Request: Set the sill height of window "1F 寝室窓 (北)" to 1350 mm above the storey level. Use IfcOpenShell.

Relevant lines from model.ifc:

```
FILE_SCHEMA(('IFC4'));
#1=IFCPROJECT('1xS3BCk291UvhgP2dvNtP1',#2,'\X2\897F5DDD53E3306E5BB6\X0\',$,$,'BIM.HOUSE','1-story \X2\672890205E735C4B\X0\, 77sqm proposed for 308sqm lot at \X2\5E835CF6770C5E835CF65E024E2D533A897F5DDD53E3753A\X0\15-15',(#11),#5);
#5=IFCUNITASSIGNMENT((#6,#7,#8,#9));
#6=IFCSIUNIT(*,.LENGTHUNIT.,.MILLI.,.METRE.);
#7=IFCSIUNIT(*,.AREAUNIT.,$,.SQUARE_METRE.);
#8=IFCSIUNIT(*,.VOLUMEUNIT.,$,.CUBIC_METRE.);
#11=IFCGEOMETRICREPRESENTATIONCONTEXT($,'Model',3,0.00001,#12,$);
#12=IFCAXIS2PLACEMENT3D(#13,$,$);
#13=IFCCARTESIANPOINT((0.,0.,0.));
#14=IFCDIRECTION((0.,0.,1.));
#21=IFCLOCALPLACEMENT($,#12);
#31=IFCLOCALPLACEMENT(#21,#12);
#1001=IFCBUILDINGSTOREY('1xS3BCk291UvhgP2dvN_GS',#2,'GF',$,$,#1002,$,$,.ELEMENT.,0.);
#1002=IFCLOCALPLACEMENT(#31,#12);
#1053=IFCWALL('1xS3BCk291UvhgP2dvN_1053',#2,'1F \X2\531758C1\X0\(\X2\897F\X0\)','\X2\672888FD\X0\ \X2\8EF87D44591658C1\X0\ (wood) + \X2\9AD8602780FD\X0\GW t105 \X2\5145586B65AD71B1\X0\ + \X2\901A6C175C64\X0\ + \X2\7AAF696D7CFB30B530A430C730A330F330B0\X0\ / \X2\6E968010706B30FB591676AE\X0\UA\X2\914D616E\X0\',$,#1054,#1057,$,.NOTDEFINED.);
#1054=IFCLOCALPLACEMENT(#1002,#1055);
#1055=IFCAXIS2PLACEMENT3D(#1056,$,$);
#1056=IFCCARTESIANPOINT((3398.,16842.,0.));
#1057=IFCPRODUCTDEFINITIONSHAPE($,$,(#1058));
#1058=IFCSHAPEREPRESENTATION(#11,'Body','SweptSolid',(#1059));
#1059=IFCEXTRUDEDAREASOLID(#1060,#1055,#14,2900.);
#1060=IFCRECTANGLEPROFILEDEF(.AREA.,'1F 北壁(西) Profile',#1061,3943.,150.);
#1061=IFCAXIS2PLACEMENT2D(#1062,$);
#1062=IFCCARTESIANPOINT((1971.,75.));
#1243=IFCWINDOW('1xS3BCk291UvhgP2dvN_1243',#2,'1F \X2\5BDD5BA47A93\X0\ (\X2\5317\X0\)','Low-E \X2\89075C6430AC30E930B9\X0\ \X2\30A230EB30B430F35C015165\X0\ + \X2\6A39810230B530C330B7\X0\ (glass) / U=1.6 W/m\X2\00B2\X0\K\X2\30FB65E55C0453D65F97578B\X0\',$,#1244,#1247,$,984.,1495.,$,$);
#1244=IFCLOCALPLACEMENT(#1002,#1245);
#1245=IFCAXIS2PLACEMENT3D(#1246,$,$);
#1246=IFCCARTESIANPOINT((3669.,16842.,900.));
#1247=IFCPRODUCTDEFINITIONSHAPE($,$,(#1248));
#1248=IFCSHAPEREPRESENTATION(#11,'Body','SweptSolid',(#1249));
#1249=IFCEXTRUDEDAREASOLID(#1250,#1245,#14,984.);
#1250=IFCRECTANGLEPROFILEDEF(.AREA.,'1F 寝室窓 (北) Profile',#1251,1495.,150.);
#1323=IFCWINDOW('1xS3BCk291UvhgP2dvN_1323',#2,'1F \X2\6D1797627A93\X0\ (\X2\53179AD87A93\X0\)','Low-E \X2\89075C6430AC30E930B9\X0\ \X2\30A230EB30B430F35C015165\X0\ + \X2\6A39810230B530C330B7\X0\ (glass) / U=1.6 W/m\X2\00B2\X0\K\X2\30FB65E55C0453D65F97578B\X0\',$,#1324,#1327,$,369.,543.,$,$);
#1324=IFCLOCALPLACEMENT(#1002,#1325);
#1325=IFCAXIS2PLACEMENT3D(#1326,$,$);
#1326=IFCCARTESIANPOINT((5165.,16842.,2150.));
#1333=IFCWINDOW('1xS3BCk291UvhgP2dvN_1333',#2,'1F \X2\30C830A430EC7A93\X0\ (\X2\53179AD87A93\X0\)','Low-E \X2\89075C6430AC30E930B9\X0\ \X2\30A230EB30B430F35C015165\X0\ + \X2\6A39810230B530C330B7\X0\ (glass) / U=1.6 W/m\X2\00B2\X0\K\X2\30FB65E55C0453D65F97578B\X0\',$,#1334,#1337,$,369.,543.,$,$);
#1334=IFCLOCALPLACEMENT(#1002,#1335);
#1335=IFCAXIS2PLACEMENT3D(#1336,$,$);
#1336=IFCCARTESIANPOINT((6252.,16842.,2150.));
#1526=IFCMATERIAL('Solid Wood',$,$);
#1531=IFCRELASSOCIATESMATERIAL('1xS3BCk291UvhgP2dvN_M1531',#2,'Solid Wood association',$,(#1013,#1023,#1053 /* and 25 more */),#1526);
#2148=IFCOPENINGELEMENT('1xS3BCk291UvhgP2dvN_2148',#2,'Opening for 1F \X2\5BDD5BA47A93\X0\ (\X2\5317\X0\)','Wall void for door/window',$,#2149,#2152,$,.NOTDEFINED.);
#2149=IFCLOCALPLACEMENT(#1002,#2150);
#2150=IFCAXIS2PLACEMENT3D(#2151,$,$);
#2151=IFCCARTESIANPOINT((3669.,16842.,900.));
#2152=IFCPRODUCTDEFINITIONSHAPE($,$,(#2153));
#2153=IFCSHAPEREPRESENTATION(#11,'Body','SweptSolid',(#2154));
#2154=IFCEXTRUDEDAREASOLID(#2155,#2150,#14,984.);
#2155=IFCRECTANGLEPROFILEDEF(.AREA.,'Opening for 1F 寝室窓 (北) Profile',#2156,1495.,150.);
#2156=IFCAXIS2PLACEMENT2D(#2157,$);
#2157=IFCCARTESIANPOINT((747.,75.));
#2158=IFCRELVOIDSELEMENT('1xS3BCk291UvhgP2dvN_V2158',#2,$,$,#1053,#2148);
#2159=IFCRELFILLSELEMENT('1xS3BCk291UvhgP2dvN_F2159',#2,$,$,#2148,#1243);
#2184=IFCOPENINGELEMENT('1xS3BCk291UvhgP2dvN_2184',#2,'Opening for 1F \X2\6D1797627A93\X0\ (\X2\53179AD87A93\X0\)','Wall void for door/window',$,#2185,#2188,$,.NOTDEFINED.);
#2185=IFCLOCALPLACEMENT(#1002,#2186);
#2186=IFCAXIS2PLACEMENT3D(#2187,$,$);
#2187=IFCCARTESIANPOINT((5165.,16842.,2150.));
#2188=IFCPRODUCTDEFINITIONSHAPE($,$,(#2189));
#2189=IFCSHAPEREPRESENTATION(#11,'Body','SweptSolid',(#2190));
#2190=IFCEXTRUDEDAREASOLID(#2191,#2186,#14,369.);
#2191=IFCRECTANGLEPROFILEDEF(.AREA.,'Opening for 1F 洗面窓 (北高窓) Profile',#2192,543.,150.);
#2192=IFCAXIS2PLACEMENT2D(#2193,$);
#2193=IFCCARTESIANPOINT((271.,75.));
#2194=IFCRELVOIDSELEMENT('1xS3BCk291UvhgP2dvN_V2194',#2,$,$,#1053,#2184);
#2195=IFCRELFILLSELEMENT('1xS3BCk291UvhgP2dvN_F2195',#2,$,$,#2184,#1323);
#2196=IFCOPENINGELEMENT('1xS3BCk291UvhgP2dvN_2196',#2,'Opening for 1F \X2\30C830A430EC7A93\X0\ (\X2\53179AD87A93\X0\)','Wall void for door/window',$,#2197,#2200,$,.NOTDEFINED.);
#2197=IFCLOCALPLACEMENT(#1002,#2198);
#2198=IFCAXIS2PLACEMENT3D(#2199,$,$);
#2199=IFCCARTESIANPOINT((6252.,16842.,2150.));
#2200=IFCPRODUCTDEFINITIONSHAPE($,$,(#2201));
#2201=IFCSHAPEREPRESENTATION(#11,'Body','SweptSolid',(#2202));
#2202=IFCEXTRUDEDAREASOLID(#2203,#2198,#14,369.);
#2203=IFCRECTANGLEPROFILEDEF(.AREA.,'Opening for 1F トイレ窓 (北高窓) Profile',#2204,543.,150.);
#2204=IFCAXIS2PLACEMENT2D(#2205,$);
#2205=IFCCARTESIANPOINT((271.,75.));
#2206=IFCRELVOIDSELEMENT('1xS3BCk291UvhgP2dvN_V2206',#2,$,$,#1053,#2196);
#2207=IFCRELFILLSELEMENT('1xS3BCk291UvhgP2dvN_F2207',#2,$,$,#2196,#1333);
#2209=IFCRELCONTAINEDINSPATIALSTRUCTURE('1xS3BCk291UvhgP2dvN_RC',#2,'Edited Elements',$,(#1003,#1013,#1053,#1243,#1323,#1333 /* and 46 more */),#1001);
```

```python
import numpy as np
import ifcopenshell
import ifcopenshell.api.geometry
import ifcopenshell.geom
import ifcopenshell.util.element
import ifcopenshell.util.placement
import ifcopenshell.util.shape
import ifcopenshell.util.unit

model = ifcopenshell.open("model.ifc")
unit_scale = ifcopenshell.util.unit.calculate_unit_scale(model)

window = model.by_id(1243)
opening = window.FillsVoids[0].RelatingOpeningElement
storey = ifcopenshell.util.element.get_container(window, ifc_class="IfcBuildingStorey")
level = ifcopenshell.util.placement.get_local_placement(storey.ObjectPlacement)[2, 3]

# The opening's origin need not be at the sill, so measure its lowest point.
shape = ifcopenshell.geom.create_shape(ifcopenshell.geom.settings(), opening)
bottom = ifcopenshell.util.shape.get_shape_bottom_elevation(shape, shape.geometry) / unit_scale
dz = level + 1.35 / unit_scale - bottom

shift = np.array([0.0, 0.0, dz])
# The window is not placed relative to its opening, so move both.
for product in (opening, window):
    matrix = ifcopenshell.util.placement.get_local_placement(product.ObjectPlacement)
    matrix[:3, 3] += shift
    ifcopenshell.api.geometry.edit_object_placement(model, product=product, matrix=matrix, is_si=False)

print(f"moved by {dz * unit_scale:+.3f} m")

model.write("model_updated.ifc")
```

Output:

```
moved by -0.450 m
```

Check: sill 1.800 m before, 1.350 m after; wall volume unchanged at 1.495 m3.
